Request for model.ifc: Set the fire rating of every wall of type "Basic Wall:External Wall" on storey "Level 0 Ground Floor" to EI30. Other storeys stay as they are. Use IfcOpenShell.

First a look at what the model holds.

```python
import ifcopenshell
import ifcopenshell.util.element

model = ifcopenshell.open("model.ifc")
print(model.schema)
storey = next(s for s in model.by_type("IfcBuildingStorey") if s.Name == "Level 0 Ground Floor")
walls = [e for e in ifcopenshell.util.element.get_decomposition(storey) if e.is_a("IfcWall")]
seen = {}
for e in walls:
    element_type = ifcopenshell.util.element.get_type(e)
    key = (element_type.Name if element_type != e and element_type else None, ifcopenshell.util.element.get_pset(e, "Pset_WallCommon", "FireRating"))
    seen[key] = seen.get(key, 0) + 1
for (name, value), count in sorted(seen.items(), key=str):
    print(count, "x", name, "|", value)
```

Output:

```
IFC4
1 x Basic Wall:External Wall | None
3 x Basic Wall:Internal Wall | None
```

```python
import ifcopenshell
import ifcopenshell.api.pset
import ifcopenshell.util.element

model = ifcopenshell.open("model.ifc")

storey = next(s for s in model.by_type("IfcBuildingStorey") if s.Name == "Level 0 Ground Floor")
walls = [e for e in ifcopenshell.util.element.get_decomposition(storey) if e.is_a("IfcWall")]

count = 0
for e in walls:
    element_type = ifcopenshell.util.element.get_type(e)
    if element_type in (None, e) or element_type.Name != "Basic Wall:External Wall":
        continue
    # add_pset returns the element's existing set when there is one.
    pset = ifcopenshell.api.pset.add_pset(model, product=e, name="Pset_WallCommon")
    ifcopenshell.api.pset.edit_pset(model, pset=pset, properties={"FireRating": "EI30"})
    count += 1

print(count, "walls updated")

model.write("model_edited.ifc")
```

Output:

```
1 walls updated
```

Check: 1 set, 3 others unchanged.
